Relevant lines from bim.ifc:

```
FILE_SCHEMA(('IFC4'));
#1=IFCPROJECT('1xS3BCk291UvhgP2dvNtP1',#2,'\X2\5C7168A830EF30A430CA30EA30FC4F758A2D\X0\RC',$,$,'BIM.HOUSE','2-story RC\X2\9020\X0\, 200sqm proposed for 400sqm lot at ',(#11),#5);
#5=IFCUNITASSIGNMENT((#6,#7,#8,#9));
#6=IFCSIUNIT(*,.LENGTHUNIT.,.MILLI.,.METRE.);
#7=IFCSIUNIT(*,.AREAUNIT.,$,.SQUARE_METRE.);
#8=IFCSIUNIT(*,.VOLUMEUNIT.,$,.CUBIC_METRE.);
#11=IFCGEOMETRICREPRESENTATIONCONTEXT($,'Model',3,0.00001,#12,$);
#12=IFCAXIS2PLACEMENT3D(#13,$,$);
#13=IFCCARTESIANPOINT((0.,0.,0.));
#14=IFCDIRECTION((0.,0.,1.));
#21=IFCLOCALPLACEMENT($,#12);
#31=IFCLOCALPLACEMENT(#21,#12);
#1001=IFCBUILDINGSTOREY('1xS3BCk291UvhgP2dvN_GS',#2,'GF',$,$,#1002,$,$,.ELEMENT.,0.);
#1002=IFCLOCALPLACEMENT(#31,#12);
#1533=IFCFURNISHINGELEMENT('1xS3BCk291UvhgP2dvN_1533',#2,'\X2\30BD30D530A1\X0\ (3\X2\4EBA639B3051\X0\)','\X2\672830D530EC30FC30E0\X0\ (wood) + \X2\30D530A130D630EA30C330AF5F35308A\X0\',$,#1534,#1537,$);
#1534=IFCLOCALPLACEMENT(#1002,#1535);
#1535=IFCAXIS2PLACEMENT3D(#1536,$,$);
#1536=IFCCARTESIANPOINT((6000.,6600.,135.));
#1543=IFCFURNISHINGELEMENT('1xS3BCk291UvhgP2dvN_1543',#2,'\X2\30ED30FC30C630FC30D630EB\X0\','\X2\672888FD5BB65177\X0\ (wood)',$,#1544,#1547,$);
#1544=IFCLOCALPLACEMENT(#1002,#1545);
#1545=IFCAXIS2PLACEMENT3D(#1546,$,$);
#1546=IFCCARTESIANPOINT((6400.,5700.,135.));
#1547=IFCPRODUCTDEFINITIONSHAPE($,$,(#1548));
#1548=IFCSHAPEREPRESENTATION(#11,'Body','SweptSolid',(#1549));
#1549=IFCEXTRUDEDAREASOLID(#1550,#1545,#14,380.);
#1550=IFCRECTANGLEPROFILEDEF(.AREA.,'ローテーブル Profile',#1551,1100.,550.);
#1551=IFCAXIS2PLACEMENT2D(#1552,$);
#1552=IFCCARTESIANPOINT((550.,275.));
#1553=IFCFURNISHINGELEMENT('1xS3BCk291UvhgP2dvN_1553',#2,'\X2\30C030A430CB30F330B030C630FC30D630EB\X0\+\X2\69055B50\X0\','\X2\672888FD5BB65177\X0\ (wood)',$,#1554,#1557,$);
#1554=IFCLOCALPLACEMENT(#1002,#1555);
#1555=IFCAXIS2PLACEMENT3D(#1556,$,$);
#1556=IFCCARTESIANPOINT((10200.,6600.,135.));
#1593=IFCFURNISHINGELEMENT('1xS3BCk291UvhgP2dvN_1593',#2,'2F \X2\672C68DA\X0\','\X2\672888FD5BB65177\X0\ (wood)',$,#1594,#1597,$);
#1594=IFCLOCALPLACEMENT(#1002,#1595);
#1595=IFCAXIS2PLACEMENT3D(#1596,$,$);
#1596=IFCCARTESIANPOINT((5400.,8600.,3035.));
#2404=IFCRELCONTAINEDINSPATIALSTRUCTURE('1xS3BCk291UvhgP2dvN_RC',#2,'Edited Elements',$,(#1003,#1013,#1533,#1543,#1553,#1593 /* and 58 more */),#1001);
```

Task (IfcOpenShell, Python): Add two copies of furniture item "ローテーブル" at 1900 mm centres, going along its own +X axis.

```python
import ifcopenshell
import ifcopenshell.api.geometry
import ifcopenshell.api.root
import ifcopenshell.util.element
import ifcopenshell.util.placement

model = ifcopenshell.open("bim.ifc")


def reuse_history(source, copy):
    """copy_class also copies each property set's owner history, people and application; keep the originals."""
    for rel in copy.IsDefinedBy:
        if rel.is_a("IfcRelDefinesByProperties") and (history := rel.RelatingPropertyDefinition.OwnerHistory):
            rel.RelatingPropertyDefinition.OwnerHistory = source.OwnerHistory
            ifcopenshell.util.element.remove_deep2(model, history)


source = model.by_guid("1xS3BCk291UvhgP2dvN_1543")
base = ifcopenshell.util.placement.get_local_placement(source.ObjectPlacement)
step = base[:3, 0] * 1900.0

for i in range(1, 3):
    copy = ifcopenshell.api.root.copy_class(model, product=source)
    copy.Representation = ifcopenshell.util.element.copy_deep(
        model, source.Representation, exclude=["IfcGeometricRepresentationContext", "IfcRepresentationMap"]
    )
    reuse_history(source, copy)
    matrix = base.copy()
    matrix[:3, 3] += i * step
    print("added at", matrix[:3, 3].round(3) + 0.0)
    ifcopenshell.api.geometry.edit_object_placement(model, product=copy, matrix=matrix, is_si=False)

model.write("bim-out.ifc")
```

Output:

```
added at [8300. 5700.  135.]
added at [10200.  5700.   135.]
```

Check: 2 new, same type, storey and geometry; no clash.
